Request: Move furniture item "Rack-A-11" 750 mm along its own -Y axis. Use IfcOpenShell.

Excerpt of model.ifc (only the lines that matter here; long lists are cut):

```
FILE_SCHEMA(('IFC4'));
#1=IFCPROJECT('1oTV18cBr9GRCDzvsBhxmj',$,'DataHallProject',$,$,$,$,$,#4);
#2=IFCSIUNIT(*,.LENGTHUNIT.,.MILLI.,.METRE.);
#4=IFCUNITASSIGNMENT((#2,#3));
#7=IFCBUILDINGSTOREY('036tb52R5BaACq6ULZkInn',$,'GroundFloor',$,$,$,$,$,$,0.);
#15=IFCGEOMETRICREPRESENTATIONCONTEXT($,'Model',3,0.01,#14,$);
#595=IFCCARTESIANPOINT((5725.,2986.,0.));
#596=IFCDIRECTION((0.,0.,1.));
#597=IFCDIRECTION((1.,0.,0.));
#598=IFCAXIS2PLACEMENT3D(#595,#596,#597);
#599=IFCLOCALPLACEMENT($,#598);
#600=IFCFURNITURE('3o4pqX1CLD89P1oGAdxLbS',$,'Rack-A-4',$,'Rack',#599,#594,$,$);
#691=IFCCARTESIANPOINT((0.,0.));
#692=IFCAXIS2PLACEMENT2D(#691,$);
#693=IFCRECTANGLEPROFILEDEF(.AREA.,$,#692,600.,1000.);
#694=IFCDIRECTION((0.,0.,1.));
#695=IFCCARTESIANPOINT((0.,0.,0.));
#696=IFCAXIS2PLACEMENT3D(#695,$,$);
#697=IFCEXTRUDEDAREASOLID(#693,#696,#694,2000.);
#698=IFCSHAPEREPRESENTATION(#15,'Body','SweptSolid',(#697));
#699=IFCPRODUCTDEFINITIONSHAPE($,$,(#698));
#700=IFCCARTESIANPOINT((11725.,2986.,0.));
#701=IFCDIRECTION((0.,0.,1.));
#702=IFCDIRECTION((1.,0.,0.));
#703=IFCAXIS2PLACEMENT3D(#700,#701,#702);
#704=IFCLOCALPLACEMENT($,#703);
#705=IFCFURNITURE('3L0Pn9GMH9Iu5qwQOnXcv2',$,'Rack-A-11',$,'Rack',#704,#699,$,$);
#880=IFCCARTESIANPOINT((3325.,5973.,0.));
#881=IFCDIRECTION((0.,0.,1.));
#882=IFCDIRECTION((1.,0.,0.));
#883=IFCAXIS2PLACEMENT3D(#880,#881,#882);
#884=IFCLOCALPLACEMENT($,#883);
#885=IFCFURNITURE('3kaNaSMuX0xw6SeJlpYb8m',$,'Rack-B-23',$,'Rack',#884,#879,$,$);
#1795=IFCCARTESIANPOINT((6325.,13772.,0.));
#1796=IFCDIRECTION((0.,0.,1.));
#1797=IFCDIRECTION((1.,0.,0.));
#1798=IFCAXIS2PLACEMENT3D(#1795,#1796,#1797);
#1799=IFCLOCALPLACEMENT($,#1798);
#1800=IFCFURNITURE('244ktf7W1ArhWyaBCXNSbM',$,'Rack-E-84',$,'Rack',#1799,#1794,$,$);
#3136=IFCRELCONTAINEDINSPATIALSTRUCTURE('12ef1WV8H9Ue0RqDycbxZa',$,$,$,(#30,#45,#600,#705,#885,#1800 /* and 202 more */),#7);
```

```python
import ifcopenshell
import ifcopenshell.api.geometry
import ifcopenshell.util.placement
import ifcopenshell.util.unit

model = ifcopenshell.open("model.ifc")
unit_scale = ifcopenshell.util.unit.calculate_unit_scale(model)

item = model.by_guid("3L0Pn9GMH9Iu5qwQOnXcv2")
matrix = ifcopenshell.util.placement.get_local_placement(item.ObjectPlacement)
matrix[:3, 3] -= matrix[:3, 1] * 0.75 / unit_scale
ifcopenshell.api.geometry.edit_object_placement(model, product=item, matrix=matrix, is_si=False)

print(ifcopenshell.util.placement.get_local_placement(item.ObjectPlacement).round(3) + 0.0)

model.write("model_updated.ifc")
```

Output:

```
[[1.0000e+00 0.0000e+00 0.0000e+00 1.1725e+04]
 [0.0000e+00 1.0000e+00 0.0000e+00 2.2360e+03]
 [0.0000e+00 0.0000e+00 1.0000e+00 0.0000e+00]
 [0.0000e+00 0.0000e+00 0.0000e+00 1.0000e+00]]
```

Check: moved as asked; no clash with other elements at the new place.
